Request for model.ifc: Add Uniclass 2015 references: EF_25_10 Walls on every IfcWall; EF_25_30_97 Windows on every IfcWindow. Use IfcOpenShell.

First a look at what the model holds.

```python
import ifcopenshell

model = ifcopenshell.open("model.ifc")
print(model.schema)
print("classifications:", [c.Name for c in model.by_type("IfcClassification")])
for ifc_class in ("IfcDoor", "IfcRoof", "IfcStair", "IfcWall", "IfcWindow"):
    print(ifc_class, len(model.by_type(ifc_class)))
```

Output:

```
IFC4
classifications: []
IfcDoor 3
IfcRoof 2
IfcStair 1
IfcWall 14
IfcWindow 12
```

```python
import ifcopenshell
import ifcopenshell.api.classification

model = ifcopenshell.open("model.ifc")

system = ifcopenshell.api.classification.add_classification(model, classification="Uniclass 2015")

codes = {
    "IfcWall": ("EF_25_10", "Walls"),
    "IfcWindow": ("EF_25_30_97", "Windows"),
}
for ifc_class, (code, name) in codes.items():
    products = model.by_type(ifc_class)
    ifcopenshell.api.classification.add_reference(
        model, products=products, classification=system, identification=code, name=name
    )
    print(code, len(products))

model.write("model_updated.ifc")
```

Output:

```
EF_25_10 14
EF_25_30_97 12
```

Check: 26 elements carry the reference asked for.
